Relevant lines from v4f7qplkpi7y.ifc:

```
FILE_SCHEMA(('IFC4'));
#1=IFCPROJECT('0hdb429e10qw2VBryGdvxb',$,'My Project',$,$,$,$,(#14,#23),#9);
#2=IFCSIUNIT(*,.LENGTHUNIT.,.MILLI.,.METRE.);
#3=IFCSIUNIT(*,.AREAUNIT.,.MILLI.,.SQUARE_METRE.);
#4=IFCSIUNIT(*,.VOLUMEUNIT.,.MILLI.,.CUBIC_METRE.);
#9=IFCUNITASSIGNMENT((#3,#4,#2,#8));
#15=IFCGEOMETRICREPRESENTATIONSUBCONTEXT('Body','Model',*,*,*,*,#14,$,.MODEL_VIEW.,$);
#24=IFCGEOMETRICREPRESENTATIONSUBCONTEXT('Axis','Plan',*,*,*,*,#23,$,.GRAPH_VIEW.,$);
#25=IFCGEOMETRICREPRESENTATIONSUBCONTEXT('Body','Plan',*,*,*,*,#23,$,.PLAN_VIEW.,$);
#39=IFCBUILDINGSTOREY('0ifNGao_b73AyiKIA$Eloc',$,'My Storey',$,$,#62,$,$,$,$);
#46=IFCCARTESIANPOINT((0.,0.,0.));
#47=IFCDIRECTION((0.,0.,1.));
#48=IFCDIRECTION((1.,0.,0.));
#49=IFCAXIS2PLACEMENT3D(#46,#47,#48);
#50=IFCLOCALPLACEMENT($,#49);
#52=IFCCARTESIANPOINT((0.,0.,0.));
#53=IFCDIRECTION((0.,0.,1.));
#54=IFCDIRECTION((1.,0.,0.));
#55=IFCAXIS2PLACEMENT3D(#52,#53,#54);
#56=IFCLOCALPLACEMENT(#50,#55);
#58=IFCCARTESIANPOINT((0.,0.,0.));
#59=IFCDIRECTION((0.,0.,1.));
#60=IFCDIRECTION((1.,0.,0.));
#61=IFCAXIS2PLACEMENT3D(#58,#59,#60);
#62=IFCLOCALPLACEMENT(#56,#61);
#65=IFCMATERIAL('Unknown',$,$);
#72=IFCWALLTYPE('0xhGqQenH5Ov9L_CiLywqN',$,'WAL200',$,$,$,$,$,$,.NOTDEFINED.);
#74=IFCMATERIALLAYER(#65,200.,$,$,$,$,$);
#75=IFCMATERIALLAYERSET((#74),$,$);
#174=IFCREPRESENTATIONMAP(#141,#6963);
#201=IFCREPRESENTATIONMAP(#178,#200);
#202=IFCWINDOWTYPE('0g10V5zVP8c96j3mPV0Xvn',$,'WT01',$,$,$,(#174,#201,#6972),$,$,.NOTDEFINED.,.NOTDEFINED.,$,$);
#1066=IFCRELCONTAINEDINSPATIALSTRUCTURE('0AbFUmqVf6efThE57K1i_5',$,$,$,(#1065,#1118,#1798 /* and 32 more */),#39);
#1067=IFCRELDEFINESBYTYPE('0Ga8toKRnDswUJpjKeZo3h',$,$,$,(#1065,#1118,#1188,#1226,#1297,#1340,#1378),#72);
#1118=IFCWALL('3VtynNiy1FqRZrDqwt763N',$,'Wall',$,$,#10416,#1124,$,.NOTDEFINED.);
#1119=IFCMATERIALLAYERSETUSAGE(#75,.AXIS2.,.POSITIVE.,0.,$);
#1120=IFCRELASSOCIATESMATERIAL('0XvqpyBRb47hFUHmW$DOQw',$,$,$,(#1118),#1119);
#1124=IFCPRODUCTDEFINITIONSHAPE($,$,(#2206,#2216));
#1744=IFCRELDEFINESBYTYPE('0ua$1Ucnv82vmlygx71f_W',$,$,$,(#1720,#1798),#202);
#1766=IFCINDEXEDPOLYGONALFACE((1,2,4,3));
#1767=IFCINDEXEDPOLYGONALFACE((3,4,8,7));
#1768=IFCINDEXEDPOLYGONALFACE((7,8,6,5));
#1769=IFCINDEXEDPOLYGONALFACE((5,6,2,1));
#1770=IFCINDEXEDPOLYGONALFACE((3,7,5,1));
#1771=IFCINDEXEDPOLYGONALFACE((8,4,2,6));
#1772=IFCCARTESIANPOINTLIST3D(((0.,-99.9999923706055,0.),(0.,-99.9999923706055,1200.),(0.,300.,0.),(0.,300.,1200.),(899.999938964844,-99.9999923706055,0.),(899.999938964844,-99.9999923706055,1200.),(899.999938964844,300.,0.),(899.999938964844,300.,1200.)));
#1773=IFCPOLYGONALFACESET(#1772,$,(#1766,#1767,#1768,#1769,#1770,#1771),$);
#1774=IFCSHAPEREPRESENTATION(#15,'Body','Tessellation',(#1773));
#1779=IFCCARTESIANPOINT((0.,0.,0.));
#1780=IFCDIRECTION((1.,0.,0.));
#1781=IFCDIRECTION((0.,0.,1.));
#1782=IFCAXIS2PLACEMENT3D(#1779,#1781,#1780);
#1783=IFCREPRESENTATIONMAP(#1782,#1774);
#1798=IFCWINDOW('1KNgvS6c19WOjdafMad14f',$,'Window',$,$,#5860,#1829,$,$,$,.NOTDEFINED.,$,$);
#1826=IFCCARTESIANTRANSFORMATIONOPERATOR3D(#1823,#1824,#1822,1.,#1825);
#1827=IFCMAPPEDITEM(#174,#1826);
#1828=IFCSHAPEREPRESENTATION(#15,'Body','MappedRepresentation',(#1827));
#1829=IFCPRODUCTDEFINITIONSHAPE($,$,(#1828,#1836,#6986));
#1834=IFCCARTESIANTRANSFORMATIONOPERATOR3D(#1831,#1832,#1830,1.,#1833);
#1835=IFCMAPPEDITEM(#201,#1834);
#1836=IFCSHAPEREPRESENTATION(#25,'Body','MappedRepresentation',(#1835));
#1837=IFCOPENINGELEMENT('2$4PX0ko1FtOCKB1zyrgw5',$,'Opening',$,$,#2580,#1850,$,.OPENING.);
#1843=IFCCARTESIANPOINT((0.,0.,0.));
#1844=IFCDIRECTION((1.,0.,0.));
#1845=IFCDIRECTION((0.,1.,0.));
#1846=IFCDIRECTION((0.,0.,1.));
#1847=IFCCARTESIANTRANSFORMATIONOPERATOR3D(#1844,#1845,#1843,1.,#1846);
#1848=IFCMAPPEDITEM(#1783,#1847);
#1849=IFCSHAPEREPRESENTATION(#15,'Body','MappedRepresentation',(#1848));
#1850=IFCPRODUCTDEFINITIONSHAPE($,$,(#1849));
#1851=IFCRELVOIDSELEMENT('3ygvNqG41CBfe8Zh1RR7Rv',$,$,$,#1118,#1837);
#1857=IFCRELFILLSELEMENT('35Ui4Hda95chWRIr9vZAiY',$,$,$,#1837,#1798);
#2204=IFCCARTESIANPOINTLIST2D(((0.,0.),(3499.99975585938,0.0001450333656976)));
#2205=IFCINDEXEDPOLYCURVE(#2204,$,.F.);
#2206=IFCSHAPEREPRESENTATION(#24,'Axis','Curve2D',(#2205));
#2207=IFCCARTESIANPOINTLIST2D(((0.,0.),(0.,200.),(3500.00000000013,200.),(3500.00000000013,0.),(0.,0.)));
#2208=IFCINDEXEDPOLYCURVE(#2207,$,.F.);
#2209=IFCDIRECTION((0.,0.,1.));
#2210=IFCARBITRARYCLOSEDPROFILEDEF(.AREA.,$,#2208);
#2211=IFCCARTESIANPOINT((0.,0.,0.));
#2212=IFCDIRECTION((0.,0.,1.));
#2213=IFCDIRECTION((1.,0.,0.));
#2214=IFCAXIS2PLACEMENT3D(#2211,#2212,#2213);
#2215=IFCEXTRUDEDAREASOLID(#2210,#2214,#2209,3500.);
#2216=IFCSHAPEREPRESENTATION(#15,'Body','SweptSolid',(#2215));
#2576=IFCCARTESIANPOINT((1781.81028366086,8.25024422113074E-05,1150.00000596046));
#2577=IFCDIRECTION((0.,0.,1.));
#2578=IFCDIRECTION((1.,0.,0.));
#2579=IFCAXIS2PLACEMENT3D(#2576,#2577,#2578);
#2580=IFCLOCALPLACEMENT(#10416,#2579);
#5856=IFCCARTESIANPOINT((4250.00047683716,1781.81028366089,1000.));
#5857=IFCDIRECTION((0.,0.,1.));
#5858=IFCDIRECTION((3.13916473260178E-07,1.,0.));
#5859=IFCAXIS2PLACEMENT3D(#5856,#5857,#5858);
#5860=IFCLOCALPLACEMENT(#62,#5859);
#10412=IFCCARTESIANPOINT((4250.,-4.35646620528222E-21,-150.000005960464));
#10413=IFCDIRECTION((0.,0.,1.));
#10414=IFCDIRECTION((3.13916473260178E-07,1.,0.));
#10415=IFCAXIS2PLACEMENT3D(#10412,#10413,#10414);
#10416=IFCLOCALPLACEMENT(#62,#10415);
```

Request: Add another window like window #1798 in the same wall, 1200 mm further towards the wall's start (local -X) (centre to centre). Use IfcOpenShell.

```python
import ifcopenshell
import ifcopenshell.api.feature
import ifcopenshell.api.geometry
import ifcopenshell.api.root
import ifcopenshell.geom
import ifcopenshell.util.element
import ifcopenshell.util.placement
import ifcopenshell.util.shape
import ifcopenshell.util.unit

model = ifcopenshell.open("v4f7qplkpi7y.ifc")
unit_scale = ifcopenshell.util.unit.calculate_unit_scale(model)
settings = ifcopenshell.geom.settings()


def volume(element):
    """Net volume in cubic metres, openings subtracted."""
    shape = ifcopenshell.geom.create_shape(settings, element)
    return ifcopenshell.util.shape.get_volume(shape.geometry)


window = model.by_id(1798)
opening = window.FillsVoids[0].RelatingOpeningElement
wall = opening.VoidsElements[0].RelatingBuildingElement
before = volume(wall)
shift = ifcopenshell.util.placement.get_local_placement(wall.ObjectPlacement)[:3, 0] * -1.2 / unit_scale

# copy_class copies the void relationship, type, container and properties, but no geometry.
new_opening = ifcopenshell.api.root.copy_class(model, product=opening)
new_opening.Representation = ifcopenshell.util.element.copy_deep(
    model, opening.Representation, exclude=["IfcGeometricRepresentationContext", "IfcRepresentationMap"]
)
new_window = ifcopenshell.api.root.copy_class(model, product=window)
new_window.Representation = ifcopenshell.util.element.copy_deep(
    model, window.Representation, exclude=["IfcGeometricRepresentationContext", "IfcRepresentationMap"]
)
ifcopenshell.api.feature.add_filling(model, opening=new_opening, element=new_window)

for old, new in ((opening, new_opening), (window, new_window)):
    matrix = ifcopenshell.util.placement.get_local_placement(old.ObjectPlacement)
    matrix[:3, 3] += shift
    ifcopenshell.api.geometry.edit_object_placement(model, product=new, matrix=matrix, is_si=False)

after = volume(wall)

print(f"wall volume {before:.3f} -> {after:.3f} m3")

model.write("v4f7qplkpi7y_rev.ifc")
```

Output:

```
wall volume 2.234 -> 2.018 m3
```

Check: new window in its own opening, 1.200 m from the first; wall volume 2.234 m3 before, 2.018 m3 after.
